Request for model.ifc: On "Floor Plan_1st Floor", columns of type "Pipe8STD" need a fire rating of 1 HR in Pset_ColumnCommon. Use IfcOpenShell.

First a look at what the model holds.

```python
import ifcopenshell
import ifcopenshell.util.element

model = ifcopenshell.open("model.ifc")
print(model.schema)
storey = next(s for s in model.by_type("IfcBuildingStorey") if s.Name == "Floor Plan_1st Floor")
columns = [e for e in ifcopenshell.util.element.get_decomposition(storey) if e.is_a("IfcColumn")]
seen = {}
for e in columns:
    element_type = ifcopenshell.util.element.get_type(e)
    key = (element_type.Name if element_type != e and element_type else None, ifcopenshell.util.element.get_pset(e, "Pset_ColumnCommon", "FireRating"))
    seen[key] = seen.get(key, 0) + 1
for (name, value), count in sorted(seen.items(), key=str):
    print(count, "x", name, "|", value)
```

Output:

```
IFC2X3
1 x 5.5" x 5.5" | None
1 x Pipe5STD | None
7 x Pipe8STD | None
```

```python
import ifcopenshell
import ifcopenshell.api.pset
import ifcopenshell.util.element

model = ifcopenshell.open("model.ifc")

storey = next(s for s in model.by_type("IfcBuildingStorey") if s.Name == "Floor Plan_1st Floor")
columns = [e for e in ifcopenshell.util.element.get_decomposition(storey) if e.is_a("IfcColumn")]

count = 0
for e in columns:
    element_type = ifcopenshell.util.element.get_type(e)
    if element_type in (None, e) or element_type.Name != "Pipe8STD":
        continue
    # add_pset returns the element's existing set when there is one.
    pset = ifcopenshell.api.pset.add_pset(model, product=e, name="Pset_ColumnCommon")
    ifcopenshell.api.pset.edit_pset(model, pset=pset, properties={"FireRating": "1 HR"})
    count += 1

print(count, "columns updated")

model.write("model_v2.ifc")
```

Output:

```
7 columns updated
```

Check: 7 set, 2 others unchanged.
